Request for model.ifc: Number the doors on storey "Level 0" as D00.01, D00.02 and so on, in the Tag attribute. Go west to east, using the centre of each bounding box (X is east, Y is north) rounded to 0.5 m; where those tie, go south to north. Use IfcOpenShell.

First a look at what the model holds.

```python
import ifcopenshell
import ifcopenshell.util.element
import ifcopenshell.util.placement

model = ifcopenshell.open("model.ifc")
print(model.schema)
storey = next(s for s in model.by_type("IfcBuildingStorey") if s.Name == "Level 0")
doors = [e for e in ifcopenshell.util.element.get_decomposition(storey) if e.is_a("IfcDoor")]
for e in sorted(doors, key=lambda e: e.id()):
    origin = ifcopenshell.util.placement.get_local_placement(e.ObjectPlacement)[:3, 3]
    print(e.id(), e.Tag, e.Name, origin.round(2) + 0.0, sep=" | ")
```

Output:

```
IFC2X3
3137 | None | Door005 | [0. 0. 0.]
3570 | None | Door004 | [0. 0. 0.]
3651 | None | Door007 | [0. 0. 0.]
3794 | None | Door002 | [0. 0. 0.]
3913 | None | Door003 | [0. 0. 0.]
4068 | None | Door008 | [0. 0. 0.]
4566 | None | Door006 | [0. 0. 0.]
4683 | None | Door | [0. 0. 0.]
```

```python
import ifcopenshell
import ifcopenshell.geom
import ifcopenshell.util.element
import ifcopenshell.util.shape

model = ifcopenshell.open("model.ifc")
settings = ifcopenshell.geom.settings()
settings.set("use-world-coords", True)


def centre(element):
    shape = ifcopenshell.geom.create_shape(settings, element)
    return ifcopenshell.util.shape.get_bbox_centroid(shape.geometry)


storey = next(s for s in model.by_type("IfcBuildingStorey") if s.Name == "Level 0")
doors = [e for e in ifcopenshell.util.element.get_decomposition(storey) if e.is_a("IfcDoor")]

# Insertion points can sit at a corner or the storey origin, so sort by the geometry (in metres).
centres = {e: centre(e) for e in doors}
doors.sort(key=lambda e: (round(centres[e][0] / 0.5), centres[e][1]))

for i, e in enumerate(doors, start=1):
    number = f"D00.{i:02d}"
    e.Tag = number
    print(e.id(), number)

model.write("model_updated.ifc")
```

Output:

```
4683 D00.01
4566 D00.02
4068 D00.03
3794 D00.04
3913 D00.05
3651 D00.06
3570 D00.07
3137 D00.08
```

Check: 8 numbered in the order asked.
